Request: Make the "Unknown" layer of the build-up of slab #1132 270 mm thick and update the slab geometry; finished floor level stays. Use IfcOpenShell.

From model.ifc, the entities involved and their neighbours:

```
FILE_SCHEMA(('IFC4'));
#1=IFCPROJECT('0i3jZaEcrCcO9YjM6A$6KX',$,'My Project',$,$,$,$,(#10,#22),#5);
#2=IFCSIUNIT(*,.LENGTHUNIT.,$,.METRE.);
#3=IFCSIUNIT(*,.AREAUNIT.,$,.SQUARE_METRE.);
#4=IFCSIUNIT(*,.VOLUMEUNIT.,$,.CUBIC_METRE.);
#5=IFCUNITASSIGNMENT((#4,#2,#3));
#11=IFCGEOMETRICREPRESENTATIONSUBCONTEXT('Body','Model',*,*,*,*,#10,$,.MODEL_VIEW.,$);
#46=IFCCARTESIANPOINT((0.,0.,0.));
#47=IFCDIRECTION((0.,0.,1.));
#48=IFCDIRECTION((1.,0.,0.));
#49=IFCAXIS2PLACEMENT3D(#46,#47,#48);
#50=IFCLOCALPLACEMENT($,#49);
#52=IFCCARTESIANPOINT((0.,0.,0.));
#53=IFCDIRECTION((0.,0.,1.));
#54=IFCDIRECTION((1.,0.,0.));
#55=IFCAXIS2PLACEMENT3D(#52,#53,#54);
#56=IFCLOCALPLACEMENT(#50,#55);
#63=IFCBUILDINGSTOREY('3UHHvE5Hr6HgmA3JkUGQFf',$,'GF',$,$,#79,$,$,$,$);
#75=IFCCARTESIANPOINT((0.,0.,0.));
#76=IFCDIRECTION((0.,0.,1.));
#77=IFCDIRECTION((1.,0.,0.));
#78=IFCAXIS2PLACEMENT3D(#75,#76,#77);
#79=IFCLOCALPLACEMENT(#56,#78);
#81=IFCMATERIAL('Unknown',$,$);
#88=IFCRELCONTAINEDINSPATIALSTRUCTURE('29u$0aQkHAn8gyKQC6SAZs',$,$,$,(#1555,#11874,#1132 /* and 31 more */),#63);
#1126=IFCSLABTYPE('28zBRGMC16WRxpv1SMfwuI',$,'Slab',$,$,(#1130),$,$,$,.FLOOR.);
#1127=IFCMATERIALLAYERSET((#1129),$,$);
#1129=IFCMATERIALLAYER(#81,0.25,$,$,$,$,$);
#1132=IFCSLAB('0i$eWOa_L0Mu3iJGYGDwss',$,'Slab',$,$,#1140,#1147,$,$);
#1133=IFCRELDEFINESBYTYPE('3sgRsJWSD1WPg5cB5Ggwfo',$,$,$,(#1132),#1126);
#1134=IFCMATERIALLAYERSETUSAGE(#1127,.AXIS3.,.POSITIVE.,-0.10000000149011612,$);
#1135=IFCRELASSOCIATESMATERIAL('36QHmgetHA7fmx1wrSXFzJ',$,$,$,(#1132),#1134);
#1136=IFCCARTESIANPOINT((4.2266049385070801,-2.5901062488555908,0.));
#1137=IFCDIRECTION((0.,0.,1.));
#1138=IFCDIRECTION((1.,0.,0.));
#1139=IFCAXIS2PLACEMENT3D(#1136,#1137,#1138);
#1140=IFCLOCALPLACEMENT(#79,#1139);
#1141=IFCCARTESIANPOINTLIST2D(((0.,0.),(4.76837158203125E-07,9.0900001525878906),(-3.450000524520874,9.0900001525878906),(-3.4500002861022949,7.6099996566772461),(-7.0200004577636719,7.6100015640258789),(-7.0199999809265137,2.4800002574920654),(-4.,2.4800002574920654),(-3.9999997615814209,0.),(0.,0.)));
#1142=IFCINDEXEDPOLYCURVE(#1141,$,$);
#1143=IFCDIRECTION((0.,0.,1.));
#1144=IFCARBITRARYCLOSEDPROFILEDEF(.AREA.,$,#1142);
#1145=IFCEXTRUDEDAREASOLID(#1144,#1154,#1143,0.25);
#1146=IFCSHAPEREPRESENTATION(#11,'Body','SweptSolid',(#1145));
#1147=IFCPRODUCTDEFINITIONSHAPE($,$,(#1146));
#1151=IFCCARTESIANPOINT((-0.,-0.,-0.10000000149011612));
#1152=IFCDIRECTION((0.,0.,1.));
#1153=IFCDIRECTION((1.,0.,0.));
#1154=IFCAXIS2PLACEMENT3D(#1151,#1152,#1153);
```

```python
import ifcopenshell
import ifcopenshell.util.element
import ifcopenshell.util.representation

model = ifcopenshell.open("model.ifc")

layer_set = model.by_id(1127)
layer = next(l for l in layer_set.MaterialLayers if l.Material and l.Material.Name == "Unknown")
change = 0.27 - layer.LayerThickness
layer.LayerThickness += change

# Geometry does not follow the layer set by itself.
slabs = [e for e in ifcopenshell.util.element.get_elements_by_material(model, layer_set) if e.is_a("IfcSlab")]
for slab in sorted(slabs, key=lambda e: e.id()):
    body = ifcopenshell.util.representation.get_representation(slab, "Model", "Body")
    solid = body.Items[0]
    old_depth = solid.Depth
    solid.Depth += change
    # Extruded upwards: lower the start of the extrusion so the top stays.
    x, y, z = solid.Position.Location.Coordinates
    solid.Position.Location = model.createIfcCartesianPoint((x, y, z - change))
    print(slab.id(), f"{old_depth:g} -> {solid.Depth:g}")

# The layers are counted up from the underside, which has moved.
for usage in {ifcopenshell.util.element.get_material(slab) for slab in slabs}:
    usage.OffsetFromReferenceLine -= change

model.write("model_edited.ifc")
```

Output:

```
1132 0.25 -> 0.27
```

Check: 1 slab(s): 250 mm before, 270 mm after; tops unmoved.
